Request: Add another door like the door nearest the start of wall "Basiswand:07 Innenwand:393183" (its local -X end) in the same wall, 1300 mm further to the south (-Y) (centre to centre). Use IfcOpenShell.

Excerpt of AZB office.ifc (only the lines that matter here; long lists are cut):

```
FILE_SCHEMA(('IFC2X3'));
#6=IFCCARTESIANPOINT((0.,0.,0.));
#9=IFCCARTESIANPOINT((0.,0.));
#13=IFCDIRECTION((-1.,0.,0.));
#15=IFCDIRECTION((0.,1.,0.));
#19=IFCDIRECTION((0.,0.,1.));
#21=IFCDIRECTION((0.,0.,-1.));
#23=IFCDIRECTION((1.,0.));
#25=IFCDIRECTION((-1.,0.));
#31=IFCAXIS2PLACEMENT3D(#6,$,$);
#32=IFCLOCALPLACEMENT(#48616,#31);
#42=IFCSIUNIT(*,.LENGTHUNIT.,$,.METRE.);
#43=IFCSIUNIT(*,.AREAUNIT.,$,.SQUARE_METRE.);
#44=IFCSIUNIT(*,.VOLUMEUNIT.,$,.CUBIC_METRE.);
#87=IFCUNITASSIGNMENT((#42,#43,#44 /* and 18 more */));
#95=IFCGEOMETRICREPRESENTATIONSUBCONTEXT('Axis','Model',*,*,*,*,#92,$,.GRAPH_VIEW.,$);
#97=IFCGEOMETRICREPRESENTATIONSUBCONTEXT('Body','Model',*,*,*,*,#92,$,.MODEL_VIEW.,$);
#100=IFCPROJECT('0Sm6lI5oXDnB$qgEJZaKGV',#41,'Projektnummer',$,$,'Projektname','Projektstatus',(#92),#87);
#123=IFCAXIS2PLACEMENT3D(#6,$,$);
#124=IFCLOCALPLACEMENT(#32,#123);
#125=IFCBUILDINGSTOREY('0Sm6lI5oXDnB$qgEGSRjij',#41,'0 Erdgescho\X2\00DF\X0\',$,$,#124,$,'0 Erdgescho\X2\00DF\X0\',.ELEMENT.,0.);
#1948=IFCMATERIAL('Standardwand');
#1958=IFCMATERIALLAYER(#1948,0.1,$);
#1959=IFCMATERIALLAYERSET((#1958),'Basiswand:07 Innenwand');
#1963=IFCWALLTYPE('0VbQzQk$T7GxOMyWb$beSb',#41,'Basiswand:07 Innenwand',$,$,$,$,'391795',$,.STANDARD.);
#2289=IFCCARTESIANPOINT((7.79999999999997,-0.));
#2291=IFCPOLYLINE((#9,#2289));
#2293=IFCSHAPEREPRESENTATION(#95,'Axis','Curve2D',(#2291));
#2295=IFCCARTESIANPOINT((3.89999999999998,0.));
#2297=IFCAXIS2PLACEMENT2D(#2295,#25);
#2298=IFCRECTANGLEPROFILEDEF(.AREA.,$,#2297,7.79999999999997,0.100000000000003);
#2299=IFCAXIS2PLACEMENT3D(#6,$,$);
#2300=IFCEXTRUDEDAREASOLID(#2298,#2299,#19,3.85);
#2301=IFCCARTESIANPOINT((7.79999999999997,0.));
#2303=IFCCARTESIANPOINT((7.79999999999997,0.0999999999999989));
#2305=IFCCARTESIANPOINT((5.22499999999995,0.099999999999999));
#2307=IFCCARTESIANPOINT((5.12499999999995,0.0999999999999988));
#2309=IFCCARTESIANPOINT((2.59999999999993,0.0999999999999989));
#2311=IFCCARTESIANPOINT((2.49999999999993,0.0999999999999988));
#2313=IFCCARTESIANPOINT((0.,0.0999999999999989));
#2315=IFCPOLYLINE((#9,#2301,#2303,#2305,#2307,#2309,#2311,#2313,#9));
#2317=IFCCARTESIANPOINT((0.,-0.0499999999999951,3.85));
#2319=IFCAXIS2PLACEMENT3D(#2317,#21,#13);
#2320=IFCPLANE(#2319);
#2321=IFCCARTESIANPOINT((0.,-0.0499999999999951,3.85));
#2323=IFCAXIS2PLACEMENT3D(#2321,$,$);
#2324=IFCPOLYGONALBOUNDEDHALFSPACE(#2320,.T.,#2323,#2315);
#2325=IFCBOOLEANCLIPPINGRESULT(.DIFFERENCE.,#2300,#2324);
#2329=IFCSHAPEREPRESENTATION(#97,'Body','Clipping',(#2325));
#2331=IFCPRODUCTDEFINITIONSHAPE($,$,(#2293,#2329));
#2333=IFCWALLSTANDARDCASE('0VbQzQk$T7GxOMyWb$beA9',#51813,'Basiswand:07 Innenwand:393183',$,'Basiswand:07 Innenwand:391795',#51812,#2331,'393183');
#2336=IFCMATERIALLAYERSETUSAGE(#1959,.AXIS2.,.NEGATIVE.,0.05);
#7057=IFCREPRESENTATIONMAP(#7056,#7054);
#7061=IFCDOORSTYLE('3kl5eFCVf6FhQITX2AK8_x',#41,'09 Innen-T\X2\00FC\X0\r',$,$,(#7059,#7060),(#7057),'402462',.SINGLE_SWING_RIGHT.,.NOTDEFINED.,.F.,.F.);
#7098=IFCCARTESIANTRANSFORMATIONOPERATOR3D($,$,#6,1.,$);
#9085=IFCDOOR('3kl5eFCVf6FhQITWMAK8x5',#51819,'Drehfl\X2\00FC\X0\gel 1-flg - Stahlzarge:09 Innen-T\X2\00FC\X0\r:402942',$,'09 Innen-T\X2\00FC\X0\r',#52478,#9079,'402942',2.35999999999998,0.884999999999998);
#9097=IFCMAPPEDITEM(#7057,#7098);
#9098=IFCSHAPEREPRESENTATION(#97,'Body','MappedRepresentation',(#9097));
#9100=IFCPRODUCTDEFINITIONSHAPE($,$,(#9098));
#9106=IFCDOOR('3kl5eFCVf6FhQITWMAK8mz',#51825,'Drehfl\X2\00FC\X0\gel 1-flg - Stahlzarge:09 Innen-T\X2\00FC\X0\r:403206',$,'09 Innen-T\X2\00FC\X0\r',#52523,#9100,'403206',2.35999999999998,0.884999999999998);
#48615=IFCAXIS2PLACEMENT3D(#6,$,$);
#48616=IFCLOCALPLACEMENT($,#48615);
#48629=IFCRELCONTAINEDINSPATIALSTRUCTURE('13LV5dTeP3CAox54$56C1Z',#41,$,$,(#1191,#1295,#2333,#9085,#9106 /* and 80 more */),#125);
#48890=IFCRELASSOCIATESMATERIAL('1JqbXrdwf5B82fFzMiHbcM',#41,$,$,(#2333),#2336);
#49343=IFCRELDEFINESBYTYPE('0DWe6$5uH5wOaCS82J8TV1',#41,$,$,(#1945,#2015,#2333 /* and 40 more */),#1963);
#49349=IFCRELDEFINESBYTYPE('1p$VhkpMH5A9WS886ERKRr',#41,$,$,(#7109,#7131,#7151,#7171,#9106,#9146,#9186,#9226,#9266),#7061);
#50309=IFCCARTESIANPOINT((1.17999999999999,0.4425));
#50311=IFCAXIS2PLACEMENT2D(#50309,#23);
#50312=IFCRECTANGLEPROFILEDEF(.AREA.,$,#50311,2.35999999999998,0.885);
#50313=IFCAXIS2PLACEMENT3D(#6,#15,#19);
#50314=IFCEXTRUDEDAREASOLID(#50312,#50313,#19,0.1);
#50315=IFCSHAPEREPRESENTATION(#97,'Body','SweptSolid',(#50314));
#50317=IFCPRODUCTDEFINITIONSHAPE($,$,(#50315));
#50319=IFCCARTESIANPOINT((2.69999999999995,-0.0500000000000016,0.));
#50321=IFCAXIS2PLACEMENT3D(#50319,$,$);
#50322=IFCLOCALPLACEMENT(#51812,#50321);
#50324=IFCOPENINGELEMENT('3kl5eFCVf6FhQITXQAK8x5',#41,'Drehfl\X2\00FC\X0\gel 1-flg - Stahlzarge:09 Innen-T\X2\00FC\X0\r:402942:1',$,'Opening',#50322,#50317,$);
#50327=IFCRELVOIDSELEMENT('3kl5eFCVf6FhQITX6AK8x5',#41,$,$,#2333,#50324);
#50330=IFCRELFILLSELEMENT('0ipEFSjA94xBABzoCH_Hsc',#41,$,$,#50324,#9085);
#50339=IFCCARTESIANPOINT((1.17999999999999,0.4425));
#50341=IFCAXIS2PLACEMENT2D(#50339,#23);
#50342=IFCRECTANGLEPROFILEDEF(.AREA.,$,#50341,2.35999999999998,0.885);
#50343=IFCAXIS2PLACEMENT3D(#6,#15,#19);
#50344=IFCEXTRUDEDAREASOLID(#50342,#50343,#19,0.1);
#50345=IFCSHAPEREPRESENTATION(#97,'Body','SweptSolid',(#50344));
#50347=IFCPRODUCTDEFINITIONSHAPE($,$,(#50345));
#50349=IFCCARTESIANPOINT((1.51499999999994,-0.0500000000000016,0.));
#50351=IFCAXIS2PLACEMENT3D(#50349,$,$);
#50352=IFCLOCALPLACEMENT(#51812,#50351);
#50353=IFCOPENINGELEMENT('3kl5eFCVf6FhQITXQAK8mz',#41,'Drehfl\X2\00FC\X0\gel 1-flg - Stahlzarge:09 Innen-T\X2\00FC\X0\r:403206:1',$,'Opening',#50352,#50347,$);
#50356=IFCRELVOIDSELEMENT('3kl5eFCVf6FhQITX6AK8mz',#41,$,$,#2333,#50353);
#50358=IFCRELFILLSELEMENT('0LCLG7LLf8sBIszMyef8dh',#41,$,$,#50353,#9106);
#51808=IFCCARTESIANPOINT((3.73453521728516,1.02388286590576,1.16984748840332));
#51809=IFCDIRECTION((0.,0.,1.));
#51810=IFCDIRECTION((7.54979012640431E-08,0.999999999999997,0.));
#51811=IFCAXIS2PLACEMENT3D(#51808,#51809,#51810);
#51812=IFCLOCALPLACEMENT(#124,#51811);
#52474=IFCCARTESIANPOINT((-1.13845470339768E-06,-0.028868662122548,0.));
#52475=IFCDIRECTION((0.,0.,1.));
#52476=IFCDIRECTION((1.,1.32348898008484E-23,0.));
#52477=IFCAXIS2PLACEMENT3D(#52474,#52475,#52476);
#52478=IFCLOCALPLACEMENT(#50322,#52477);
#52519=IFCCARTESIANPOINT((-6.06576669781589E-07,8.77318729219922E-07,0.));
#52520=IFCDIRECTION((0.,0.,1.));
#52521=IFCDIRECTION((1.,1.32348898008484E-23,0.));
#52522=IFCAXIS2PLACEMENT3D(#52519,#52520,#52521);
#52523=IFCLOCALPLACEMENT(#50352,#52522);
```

```python
import ifcopenshell
import ifcopenshell.api.feature
import ifcopenshell.api.geometry
import ifcopenshell.api.root
import ifcopenshell.geom
import ifcopenshell.util.element
import ifcopenshell.util.placement
import ifcopenshell.util.shape

model = ifcopenshell.open("AZB office.ifc")
settings = ifcopenshell.geom.settings()


def volume(element):
    """Net volume in cubic metres, openings subtracted."""
    shape = ifcopenshell.geom.create_shape(settings, element)
    return ifcopenshell.util.shape.get_volume(shape.geometry)


def reuse_history(source, copy):
    """copy_class also copies each property set's owner history, people and application; keep the originals."""
    for rel in copy.IsDefinedBy:
        if rel.is_a("IfcRelDefinesByProperties") and (history := rel.RelatingPropertyDefinition.OwnerHistory):
            rel.RelatingPropertyDefinition.OwnerHistory = source.OwnerHistory
            ifcopenshell.util.element.remove_deep2(model, history)


door = model.by_id(9106)
opening = door.FillsVoids[0].RelatingOpeningElement
wall = opening.VoidsElements[0].RelatingBuildingElement
before = volume(wall)
shift = ifcopenshell.util.placement.get_local_placement(wall.ObjectPlacement)[:3, 0] * -1.3

# copy_class copies the void relationship, type, container and properties, but no geometry.
new_opening = ifcopenshell.api.root.copy_class(model, product=opening)
new_opening.Representation = ifcopenshell.util.element.copy_deep(
    model, opening.Representation, exclude=["IfcGeometricRepresentationContext", "IfcRepresentationMap"]
)
new_opening.Name = "Drehflügel 1-flg - Stahlzarge:09 Innen-Tür"
new_door = ifcopenshell.api.root.copy_class(model, product=door)
new_door.Representation = ifcopenshell.util.element.copy_deep(
    model, door.Representation, exclude=["IfcGeometricRepresentationContext", "IfcRepresentationMap"]
)
new_door.Name = "Drehflügel 1-flg - Stahlzarge:09 Innen-Tür"
new_door.Tag = None
reuse_history(door, new_door)
fills = ifcopenshell.api.feature.add_filling(model, opening=new_opening, element=new_door)
fills.OwnerHistory = new_door.OwnerHistory  # required in IFC2X3

for old, new in ((opening, new_opening), (door, new_door)):
    matrix = ifcopenshell.util.placement.get_local_placement(old.ObjectPlacement)
    matrix[:3, 3] += shift
    ifcopenshell.api.geometry.edit_object_placement(model, product=new, matrix=matrix, is_si=False)

after = volume(wall)

print(f"wall volume {before:.3f} -> {after:.3f} m3")

model.write("AZB office_rev.ifc")
```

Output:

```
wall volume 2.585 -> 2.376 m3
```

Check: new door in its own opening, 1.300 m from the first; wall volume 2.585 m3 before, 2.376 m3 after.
